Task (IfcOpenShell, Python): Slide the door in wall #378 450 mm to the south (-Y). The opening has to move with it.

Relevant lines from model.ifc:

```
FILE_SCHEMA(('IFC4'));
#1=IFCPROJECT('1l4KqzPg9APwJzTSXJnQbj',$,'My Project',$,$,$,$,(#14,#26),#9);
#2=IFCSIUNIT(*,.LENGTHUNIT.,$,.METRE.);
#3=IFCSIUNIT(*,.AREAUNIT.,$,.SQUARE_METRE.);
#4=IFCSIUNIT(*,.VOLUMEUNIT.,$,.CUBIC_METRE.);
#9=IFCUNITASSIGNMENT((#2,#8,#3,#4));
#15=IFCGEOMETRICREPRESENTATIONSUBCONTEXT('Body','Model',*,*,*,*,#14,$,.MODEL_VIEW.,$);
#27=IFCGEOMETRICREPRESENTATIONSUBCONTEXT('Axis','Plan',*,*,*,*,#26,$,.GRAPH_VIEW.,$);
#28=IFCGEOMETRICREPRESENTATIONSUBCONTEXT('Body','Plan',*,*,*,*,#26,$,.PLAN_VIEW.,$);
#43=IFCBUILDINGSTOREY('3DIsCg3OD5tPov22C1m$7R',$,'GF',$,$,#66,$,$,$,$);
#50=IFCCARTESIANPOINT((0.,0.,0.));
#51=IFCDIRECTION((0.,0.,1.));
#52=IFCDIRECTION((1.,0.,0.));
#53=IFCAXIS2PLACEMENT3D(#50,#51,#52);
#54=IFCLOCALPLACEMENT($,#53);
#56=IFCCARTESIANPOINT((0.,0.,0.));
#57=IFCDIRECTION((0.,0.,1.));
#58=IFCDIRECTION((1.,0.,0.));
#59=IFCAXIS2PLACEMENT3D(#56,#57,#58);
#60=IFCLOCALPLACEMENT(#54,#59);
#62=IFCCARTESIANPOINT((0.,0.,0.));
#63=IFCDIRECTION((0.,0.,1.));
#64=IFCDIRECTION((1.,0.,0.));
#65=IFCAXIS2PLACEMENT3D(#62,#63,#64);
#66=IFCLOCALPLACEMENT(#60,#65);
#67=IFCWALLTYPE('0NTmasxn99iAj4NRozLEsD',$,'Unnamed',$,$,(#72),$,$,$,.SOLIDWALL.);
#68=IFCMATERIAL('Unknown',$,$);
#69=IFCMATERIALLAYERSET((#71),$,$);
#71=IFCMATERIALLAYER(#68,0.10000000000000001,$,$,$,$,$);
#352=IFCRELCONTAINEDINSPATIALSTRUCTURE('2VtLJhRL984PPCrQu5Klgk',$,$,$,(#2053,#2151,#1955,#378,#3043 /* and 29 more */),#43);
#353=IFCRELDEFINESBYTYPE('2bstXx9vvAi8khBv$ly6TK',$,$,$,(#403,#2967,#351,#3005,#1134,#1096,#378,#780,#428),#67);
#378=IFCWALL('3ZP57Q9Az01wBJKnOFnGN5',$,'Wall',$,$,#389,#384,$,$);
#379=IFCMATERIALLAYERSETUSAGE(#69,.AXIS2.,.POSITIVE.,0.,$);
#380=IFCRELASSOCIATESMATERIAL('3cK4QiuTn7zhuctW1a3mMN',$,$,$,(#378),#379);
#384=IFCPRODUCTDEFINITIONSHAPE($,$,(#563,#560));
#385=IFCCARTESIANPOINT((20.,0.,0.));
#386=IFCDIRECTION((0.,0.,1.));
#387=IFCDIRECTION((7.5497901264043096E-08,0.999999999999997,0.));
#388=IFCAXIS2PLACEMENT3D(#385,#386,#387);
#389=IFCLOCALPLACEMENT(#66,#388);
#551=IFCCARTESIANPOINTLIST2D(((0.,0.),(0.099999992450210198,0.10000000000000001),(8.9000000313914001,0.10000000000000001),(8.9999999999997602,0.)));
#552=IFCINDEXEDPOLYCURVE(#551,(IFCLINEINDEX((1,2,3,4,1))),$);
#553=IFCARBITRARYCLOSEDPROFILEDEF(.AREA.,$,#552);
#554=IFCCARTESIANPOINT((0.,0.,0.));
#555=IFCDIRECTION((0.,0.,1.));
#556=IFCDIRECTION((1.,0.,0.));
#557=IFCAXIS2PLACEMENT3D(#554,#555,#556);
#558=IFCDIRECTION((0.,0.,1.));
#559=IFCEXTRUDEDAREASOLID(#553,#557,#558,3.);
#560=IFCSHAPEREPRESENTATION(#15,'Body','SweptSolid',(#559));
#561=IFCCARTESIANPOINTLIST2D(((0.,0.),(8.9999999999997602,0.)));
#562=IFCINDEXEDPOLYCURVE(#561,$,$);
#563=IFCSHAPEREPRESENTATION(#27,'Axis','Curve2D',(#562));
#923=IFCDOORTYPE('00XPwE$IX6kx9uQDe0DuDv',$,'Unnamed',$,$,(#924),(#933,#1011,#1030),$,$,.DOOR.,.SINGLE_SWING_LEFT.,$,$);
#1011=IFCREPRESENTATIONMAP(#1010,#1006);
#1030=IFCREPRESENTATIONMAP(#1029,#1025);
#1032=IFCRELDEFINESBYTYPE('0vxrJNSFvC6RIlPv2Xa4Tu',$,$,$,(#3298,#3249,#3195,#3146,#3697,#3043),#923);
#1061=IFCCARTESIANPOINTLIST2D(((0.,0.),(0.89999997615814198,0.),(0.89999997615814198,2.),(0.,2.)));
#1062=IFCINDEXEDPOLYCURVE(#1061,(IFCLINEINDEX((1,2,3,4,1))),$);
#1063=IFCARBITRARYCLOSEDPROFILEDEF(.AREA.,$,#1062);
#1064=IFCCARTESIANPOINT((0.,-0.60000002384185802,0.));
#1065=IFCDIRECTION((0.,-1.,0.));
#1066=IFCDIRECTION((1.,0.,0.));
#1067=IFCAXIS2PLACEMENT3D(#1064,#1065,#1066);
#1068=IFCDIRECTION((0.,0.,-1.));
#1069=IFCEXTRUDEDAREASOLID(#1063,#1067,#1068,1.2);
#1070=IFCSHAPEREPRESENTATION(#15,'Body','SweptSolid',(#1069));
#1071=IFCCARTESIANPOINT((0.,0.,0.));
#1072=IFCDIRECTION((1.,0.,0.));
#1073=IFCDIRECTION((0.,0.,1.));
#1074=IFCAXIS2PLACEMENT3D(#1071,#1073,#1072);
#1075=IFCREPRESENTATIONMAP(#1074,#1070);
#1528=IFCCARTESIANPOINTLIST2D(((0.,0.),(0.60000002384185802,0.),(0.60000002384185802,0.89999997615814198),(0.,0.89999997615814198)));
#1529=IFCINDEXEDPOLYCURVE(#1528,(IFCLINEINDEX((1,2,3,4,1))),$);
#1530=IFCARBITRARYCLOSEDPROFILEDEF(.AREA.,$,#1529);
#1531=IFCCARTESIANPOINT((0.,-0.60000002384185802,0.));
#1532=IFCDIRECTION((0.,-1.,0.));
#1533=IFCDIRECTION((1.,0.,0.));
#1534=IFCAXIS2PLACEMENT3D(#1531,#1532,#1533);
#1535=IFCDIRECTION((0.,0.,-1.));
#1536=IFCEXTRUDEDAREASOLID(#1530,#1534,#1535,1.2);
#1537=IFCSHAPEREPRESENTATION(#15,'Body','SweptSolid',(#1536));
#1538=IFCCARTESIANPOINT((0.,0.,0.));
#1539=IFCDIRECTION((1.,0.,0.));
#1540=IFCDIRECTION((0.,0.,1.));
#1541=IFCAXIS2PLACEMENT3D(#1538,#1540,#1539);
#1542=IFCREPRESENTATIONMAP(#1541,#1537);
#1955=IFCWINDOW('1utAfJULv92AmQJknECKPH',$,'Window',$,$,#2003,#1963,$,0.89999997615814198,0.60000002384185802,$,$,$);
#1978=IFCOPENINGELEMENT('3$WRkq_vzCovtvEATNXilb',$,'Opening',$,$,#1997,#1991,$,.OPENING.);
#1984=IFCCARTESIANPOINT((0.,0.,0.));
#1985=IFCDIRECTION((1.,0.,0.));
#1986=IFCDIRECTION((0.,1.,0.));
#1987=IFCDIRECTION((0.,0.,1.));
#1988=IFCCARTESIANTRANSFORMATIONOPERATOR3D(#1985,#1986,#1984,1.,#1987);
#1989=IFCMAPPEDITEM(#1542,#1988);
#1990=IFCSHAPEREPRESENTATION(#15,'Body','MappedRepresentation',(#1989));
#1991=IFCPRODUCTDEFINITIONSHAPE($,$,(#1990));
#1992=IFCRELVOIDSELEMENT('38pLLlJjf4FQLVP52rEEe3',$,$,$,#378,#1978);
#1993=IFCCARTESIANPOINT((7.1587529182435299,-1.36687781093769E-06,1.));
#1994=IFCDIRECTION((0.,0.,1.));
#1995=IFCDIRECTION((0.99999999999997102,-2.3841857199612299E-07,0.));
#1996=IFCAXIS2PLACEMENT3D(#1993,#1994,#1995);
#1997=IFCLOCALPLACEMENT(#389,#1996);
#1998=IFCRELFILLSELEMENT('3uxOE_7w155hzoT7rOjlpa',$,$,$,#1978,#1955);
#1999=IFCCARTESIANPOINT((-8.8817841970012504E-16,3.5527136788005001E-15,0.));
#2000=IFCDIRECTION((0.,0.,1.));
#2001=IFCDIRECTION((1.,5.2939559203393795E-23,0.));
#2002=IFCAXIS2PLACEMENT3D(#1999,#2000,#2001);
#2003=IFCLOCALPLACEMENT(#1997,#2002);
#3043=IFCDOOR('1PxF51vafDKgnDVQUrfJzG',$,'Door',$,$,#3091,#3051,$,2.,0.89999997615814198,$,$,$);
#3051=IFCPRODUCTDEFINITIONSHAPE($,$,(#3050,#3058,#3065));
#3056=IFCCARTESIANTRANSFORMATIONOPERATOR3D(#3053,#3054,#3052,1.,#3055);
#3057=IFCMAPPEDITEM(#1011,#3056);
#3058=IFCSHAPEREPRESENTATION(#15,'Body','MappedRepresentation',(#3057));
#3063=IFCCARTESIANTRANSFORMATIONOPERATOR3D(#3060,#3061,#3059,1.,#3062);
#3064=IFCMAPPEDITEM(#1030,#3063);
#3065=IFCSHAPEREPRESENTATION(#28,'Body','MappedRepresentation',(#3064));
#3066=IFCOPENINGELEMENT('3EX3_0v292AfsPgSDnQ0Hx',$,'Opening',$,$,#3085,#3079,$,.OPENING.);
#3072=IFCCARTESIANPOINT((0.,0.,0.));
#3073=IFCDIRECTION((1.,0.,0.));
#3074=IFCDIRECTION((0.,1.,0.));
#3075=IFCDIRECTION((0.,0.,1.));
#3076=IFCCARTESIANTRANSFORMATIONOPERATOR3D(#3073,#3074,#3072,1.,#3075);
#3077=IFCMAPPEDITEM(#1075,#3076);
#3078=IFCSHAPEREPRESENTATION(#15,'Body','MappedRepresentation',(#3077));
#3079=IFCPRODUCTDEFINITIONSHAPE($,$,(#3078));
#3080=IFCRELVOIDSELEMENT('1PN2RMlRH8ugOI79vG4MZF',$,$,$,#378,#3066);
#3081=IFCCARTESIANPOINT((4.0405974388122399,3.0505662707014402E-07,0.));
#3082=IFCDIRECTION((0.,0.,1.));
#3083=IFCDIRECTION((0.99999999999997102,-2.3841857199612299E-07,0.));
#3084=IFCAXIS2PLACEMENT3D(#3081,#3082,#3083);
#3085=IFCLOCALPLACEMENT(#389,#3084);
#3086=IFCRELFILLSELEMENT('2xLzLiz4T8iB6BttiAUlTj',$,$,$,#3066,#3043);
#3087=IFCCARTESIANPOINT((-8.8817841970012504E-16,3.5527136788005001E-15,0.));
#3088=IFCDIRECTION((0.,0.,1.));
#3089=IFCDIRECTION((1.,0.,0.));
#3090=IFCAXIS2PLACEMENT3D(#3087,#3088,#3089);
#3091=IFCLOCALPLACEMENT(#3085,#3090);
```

```python
import ifcopenshell
import ifcopenshell.api.geometry
import ifcopenshell.util.placement

model = ifcopenshell.open("model.ifc")

door = model.by_id(3043)
opening = door.FillsVoids[0].RelatingOpeningElement
wall = opening.VoidsElements[0].RelatingBuildingElement

wall_matrix = ifcopenshell.util.placement.get_local_placement(wall.ObjectPlacement)
shift = wall_matrix[:3, 0] * -0.45
before = ifcopenshell.util.placement.get_local_placement(door.ObjectPlacement)[:3, 3].copy()

# The door is placed relative to its opening, so it follows when the opening moves.
matrix = ifcopenshell.util.placement.get_local_placement(opening.ObjectPlacement)
matrix[:3, 3] += shift
ifcopenshell.api.geometry.edit_object_placement(
    model, product=opening, matrix=matrix, is_si=False, should_transform_children=True
)

after = ifcopenshell.util.placement.get_local_placement(door.ObjectPlacement)[:3, 3]
print("door moved by", (after - before).round(3) + 0.0)

model.write("model-out.ifc")
```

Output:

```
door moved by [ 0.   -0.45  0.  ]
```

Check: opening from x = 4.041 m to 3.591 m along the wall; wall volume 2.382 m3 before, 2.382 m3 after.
